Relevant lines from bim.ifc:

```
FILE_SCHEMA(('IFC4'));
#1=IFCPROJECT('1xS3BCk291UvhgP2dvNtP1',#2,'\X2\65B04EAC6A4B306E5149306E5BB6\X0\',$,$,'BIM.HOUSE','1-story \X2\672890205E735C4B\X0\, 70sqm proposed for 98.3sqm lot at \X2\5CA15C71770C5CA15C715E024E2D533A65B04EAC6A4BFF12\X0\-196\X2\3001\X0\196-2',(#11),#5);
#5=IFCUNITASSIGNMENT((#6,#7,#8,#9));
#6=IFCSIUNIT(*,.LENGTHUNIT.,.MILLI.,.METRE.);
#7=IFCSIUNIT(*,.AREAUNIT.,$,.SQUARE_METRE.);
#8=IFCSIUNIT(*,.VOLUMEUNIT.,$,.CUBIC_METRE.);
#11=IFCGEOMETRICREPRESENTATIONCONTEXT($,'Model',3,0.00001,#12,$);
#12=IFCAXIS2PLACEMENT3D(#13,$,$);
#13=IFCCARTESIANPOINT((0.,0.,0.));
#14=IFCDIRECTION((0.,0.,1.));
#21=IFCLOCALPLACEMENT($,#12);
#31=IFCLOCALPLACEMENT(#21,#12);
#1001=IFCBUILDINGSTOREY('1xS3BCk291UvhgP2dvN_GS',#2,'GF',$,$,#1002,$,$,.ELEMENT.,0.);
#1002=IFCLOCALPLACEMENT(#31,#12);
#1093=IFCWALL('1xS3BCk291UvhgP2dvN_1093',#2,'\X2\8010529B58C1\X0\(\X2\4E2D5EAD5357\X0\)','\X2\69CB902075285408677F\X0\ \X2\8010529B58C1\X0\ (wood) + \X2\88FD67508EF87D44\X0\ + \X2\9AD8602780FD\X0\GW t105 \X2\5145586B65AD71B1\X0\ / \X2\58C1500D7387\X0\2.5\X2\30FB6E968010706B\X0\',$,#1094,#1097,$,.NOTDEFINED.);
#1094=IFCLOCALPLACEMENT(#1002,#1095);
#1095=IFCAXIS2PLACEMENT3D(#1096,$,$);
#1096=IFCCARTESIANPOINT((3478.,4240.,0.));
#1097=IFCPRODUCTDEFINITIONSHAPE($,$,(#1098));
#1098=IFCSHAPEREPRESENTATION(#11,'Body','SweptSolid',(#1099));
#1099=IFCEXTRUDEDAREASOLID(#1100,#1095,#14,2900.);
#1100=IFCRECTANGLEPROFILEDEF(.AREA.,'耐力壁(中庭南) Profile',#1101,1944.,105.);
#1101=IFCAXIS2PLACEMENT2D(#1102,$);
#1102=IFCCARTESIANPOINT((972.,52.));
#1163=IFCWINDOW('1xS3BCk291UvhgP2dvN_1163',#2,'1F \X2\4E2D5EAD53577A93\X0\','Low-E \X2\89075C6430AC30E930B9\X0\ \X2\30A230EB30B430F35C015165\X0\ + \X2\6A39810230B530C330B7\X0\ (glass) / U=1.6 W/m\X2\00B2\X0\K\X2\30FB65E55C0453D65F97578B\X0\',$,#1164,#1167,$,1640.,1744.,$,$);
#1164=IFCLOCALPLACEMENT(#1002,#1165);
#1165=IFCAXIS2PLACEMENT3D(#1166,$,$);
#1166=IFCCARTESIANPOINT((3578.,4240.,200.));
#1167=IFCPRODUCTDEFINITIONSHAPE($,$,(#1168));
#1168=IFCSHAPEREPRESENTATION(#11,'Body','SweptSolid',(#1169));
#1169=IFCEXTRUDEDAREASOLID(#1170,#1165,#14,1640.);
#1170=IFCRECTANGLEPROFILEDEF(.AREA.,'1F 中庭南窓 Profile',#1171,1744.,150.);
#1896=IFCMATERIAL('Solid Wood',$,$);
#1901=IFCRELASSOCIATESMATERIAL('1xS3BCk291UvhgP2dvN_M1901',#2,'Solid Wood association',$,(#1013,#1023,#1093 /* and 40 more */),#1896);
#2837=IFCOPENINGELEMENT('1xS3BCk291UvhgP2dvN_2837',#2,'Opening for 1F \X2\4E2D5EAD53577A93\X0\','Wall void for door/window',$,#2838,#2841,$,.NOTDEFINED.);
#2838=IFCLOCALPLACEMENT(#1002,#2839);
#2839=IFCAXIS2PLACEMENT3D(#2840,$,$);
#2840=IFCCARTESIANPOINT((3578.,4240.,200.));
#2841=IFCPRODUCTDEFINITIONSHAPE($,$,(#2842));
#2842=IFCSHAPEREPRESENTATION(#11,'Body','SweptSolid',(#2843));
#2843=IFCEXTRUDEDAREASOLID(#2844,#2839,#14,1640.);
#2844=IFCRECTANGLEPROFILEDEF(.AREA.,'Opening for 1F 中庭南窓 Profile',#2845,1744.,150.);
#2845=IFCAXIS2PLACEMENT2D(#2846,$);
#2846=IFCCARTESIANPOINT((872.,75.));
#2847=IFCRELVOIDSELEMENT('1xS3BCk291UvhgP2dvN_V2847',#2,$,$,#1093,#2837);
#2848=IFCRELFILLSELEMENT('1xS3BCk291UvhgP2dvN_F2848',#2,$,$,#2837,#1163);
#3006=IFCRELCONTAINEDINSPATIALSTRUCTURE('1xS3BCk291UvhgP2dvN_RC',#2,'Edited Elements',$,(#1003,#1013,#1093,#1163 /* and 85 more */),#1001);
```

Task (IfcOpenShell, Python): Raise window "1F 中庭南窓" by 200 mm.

```python
import numpy as np
import ifcopenshell
import ifcopenshell.api.geometry
import ifcopenshell.util.placement
import ifcopenshell.util.unit

model = ifcopenshell.open("bim.ifc")
unit_scale = ifcopenshell.util.unit.calculate_unit_scale(model)

window = model.by_guid("1xS3BCk291UvhgP2dvN_1163")
opening = window.FillsVoids[0].RelatingOpeningElement
dz = 200.0

shift = np.array([0.0, 0.0, dz])
# The window is not placed relative to its opening, so move both.
for product in (opening, window):
    matrix = ifcopenshell.util.placement.get_local_placement(product.ObjectPlacement)
    matrix[:3, 3] += shift
    ifcopenshell.api.geometry.edit_object_placement(model, product=product, matrix=matrix, is_si=False)

print(f"moved by {dz * unit_scale:+.3f} m")

model.write("bim-out.ifc")
```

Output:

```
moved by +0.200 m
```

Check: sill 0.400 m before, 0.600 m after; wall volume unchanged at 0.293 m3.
